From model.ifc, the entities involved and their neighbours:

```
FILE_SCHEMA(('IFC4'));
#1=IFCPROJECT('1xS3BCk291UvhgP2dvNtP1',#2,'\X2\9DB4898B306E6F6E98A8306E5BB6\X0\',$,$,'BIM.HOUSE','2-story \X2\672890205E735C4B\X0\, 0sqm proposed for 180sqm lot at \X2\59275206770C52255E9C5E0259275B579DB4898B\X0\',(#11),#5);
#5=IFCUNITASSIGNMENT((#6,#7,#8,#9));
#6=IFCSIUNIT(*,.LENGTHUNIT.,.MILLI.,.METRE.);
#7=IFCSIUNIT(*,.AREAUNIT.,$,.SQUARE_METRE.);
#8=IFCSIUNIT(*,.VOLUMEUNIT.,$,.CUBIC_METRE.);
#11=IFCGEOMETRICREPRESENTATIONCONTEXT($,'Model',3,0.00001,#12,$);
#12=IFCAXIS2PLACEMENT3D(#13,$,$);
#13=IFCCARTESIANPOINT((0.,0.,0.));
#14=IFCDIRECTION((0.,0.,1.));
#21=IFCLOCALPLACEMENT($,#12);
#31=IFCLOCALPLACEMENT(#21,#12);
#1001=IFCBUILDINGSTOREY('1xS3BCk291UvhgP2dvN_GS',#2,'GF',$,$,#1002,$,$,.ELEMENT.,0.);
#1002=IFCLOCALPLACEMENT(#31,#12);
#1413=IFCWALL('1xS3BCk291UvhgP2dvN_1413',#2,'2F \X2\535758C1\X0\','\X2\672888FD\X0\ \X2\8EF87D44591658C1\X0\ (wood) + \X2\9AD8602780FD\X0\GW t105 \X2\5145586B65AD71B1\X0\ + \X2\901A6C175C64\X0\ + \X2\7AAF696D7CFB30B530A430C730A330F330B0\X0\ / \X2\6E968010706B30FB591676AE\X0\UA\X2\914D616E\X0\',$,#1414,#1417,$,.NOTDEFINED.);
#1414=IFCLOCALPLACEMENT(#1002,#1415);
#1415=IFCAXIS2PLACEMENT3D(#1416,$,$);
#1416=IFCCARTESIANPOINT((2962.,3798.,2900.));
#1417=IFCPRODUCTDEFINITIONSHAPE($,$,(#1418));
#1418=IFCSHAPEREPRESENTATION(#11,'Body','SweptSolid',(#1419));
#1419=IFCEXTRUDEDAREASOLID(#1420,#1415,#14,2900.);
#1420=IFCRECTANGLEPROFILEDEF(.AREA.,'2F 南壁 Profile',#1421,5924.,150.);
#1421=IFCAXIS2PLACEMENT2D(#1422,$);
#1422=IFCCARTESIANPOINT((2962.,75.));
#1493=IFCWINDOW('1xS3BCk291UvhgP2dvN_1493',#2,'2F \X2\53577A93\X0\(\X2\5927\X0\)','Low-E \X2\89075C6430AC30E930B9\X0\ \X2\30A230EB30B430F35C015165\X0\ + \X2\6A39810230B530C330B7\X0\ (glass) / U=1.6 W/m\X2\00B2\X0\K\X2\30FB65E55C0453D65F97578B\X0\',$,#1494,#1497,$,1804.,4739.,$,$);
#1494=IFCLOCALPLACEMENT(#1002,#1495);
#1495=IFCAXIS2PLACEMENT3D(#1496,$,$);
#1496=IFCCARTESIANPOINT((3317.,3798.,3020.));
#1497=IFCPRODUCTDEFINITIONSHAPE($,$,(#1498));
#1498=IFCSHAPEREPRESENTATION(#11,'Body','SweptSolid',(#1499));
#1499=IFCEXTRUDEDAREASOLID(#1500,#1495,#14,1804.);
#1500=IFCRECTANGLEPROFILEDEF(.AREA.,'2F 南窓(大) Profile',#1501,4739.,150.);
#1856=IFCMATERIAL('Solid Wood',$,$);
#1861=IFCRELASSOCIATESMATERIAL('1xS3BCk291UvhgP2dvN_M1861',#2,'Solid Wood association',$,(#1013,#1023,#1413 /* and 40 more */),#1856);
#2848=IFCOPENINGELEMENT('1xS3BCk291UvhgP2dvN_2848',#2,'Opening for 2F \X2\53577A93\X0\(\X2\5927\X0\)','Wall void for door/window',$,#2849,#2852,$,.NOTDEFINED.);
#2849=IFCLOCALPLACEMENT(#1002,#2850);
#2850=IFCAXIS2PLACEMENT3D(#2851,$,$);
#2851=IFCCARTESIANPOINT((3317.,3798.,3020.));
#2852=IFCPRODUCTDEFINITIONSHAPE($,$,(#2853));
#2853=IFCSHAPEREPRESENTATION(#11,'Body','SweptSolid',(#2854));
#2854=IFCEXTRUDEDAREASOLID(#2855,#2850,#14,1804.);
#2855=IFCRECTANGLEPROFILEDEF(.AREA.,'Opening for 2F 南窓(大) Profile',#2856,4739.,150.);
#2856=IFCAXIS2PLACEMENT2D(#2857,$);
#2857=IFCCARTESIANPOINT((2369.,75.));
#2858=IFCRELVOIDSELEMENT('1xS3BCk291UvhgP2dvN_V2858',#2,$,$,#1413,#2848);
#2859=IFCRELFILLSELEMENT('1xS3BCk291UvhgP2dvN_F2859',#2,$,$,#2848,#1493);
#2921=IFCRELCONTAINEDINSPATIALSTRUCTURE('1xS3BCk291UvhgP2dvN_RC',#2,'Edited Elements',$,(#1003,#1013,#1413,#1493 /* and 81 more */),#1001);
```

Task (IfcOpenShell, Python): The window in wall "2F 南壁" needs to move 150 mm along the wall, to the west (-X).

```python
import ifcopenshell
import ifcopenshell.api.geometry
import ifcopenshell.util.placement

model = ifcopenshell.open("model.ifc")

window = model.by_id(1493)
opening = window.FillsVoids[0].RelatingOpeningElement
wall = opening.VoidsElements[0].RelatingBuildingElement

wall_matrix = ifcopenshell.util.placement.get_local_placement(wall.ObjectPlacement)
shift = wall_matrix[:3, 0] * -150.0
before = ifcopenshell.util.placement.get_local_placement(window.ObjectPlacement)[:3, 3].copy()

# The window is not placed relative to its opening, so move both.
for product in (opening, window):
    matrix = ifcopenshell.util.placement.get_local_placement(product.ObjectPlacement)
    matrix[:3, 3] += shift
    ifcopenshell.api.geometry.edit_object_placement(model, product=product, matrix=matrix, is_si=False)

after = ifcopenshell.util.placement.get_local_placement(window.ObjectPlacement)[:3, 3]
print("window moved by", (after - before).round(3) + 0.0)

model.write("model_updated.ifc")
```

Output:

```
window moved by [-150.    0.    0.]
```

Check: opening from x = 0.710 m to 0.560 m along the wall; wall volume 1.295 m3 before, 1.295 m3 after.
